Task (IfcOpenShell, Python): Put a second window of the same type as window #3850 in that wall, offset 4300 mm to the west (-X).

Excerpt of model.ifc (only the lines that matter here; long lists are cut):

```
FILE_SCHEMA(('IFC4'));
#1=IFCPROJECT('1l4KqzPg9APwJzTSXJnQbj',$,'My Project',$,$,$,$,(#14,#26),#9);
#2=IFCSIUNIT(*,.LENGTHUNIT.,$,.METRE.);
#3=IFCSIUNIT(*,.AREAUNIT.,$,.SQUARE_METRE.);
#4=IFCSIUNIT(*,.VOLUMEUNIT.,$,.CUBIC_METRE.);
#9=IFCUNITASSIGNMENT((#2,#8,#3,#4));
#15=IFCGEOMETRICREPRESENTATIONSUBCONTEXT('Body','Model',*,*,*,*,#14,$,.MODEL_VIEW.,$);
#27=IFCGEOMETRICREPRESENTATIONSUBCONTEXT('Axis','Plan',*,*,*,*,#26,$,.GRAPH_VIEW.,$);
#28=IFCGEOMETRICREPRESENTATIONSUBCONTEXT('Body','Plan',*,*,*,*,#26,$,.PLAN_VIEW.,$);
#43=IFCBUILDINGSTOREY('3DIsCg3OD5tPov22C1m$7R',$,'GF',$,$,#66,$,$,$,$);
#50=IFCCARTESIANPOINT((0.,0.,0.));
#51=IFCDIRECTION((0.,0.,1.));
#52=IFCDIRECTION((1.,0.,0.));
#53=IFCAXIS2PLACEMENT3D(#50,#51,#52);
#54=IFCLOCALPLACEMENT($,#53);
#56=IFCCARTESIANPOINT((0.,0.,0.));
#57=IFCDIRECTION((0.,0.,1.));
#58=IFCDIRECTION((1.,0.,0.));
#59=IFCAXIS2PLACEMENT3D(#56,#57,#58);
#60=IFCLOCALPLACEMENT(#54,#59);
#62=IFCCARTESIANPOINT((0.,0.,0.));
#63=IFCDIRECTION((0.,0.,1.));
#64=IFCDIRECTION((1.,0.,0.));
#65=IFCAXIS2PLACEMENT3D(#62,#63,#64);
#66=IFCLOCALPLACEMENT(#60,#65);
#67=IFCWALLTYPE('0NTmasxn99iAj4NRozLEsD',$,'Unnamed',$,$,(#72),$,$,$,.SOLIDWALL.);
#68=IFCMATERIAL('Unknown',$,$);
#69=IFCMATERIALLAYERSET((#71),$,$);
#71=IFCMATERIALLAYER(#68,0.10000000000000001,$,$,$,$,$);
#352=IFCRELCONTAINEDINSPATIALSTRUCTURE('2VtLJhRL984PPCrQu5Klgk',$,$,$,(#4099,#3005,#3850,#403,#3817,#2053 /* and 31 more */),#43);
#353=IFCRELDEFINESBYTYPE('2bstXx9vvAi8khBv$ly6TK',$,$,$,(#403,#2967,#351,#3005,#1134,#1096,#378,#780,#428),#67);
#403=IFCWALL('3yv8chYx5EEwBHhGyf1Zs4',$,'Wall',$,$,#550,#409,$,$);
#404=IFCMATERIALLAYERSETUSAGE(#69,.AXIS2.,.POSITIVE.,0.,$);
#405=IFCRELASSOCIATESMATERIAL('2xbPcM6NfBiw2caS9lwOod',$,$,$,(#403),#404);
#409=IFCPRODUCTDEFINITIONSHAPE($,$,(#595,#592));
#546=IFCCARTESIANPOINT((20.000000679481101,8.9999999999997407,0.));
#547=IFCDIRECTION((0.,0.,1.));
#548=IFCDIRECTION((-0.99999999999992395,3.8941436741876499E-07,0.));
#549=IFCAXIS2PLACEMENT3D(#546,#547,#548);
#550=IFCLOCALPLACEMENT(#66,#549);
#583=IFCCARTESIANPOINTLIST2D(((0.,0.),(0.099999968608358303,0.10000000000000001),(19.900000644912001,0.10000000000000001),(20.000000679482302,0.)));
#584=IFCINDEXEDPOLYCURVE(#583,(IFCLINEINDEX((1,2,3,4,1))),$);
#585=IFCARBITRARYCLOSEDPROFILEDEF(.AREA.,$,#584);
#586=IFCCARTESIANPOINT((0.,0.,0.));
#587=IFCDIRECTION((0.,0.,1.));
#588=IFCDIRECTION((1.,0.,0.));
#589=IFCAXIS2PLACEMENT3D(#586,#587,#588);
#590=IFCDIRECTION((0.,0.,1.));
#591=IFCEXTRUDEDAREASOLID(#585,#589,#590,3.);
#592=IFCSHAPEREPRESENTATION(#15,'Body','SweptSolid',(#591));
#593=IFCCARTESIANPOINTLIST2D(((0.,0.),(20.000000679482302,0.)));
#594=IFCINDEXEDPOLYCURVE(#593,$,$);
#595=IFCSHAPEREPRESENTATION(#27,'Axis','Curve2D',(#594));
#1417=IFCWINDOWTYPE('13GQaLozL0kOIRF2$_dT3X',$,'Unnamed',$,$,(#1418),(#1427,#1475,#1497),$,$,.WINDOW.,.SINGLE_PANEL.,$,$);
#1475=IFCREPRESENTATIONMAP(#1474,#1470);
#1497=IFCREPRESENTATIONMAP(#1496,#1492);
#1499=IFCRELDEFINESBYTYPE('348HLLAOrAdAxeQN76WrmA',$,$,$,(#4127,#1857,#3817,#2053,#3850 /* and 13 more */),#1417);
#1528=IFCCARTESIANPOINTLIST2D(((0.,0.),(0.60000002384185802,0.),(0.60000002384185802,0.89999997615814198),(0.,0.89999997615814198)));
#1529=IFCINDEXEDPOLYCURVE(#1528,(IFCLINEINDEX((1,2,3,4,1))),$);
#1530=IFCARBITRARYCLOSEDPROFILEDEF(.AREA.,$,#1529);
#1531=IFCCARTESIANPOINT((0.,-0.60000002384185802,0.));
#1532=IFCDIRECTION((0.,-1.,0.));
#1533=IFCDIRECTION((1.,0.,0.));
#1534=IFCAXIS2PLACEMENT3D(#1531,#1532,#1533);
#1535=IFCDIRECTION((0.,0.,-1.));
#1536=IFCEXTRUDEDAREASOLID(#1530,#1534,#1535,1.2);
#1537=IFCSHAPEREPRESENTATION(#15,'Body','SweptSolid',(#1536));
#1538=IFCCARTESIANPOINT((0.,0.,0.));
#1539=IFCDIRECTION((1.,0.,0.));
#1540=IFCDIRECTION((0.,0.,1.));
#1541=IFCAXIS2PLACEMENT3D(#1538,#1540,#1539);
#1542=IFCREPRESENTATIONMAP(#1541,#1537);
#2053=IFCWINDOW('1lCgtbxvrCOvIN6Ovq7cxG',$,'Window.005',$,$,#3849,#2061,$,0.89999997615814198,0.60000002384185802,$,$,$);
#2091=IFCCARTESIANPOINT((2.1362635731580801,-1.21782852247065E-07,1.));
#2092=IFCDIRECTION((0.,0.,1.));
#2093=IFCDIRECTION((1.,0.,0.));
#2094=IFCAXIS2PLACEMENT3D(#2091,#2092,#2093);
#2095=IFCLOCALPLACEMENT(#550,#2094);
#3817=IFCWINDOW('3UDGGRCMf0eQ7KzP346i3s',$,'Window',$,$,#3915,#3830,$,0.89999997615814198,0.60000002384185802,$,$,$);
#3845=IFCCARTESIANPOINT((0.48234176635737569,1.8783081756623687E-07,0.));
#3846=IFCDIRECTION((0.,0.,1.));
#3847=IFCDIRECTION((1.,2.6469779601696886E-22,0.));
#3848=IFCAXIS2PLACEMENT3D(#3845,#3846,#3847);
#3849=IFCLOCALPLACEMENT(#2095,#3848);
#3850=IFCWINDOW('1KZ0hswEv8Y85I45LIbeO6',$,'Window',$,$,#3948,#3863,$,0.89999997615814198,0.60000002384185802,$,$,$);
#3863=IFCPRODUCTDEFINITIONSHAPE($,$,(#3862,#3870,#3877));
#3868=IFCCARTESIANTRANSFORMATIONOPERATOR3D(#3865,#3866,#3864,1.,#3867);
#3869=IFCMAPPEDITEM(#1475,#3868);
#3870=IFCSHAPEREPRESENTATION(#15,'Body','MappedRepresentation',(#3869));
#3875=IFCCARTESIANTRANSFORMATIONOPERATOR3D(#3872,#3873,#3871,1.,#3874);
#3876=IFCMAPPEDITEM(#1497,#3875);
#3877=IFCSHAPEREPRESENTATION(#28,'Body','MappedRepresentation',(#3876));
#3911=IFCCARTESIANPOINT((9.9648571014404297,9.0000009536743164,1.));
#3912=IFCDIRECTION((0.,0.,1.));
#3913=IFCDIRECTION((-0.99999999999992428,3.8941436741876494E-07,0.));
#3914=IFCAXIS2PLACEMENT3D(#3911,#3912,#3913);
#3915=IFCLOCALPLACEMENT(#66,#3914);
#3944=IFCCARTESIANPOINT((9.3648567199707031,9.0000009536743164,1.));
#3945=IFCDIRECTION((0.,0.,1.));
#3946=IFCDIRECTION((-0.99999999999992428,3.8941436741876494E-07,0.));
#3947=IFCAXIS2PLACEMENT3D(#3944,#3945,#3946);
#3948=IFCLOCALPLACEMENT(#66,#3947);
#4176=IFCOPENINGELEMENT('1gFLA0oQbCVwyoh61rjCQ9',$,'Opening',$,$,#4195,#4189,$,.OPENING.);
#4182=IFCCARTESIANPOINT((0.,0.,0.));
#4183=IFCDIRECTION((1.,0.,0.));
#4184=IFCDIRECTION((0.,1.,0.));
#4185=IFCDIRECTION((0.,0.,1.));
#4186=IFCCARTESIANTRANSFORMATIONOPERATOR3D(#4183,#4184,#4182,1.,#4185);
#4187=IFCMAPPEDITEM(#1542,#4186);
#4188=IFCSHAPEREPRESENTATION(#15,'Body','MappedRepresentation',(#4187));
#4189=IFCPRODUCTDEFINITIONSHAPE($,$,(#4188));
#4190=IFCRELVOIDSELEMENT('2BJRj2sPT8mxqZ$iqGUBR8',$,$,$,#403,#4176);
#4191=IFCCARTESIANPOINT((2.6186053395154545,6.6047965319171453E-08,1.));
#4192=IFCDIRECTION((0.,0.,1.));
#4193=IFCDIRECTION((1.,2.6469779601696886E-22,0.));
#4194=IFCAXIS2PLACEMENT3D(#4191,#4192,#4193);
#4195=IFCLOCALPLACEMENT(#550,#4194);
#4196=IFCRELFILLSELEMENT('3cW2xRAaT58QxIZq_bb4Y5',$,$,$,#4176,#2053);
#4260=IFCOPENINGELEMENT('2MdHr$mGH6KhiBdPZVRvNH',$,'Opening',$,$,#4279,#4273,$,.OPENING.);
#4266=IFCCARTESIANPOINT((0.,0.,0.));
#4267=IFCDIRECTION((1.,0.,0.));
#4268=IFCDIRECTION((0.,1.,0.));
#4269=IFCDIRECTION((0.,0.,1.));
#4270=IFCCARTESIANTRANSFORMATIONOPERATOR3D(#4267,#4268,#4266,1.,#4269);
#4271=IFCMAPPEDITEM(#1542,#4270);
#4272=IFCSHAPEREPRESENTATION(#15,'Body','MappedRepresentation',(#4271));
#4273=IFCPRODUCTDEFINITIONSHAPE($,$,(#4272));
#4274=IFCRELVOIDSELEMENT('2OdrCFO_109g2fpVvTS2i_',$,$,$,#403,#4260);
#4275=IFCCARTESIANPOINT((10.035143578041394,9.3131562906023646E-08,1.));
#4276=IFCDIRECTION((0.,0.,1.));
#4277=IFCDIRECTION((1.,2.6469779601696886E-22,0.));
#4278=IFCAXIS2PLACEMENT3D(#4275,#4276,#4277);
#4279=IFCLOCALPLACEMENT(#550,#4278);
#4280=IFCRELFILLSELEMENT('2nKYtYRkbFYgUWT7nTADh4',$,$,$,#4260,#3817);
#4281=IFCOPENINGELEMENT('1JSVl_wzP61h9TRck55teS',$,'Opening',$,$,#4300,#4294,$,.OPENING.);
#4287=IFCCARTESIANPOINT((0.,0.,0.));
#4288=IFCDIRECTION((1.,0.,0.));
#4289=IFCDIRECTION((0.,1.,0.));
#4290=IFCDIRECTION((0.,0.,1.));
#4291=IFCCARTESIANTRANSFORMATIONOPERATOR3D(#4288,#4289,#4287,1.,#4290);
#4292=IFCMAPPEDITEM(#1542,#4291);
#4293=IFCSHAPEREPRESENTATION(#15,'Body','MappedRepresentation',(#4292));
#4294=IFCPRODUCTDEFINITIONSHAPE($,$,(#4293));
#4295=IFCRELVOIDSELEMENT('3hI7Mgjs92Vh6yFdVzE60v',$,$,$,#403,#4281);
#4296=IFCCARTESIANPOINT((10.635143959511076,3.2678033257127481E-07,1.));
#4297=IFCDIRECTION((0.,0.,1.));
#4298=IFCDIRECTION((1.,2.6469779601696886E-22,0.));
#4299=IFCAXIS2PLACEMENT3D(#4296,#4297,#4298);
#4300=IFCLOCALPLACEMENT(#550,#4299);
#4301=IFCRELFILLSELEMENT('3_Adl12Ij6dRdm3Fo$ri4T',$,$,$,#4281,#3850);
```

```python
import ifcopenshell
import ifcopenshell.api.feature
import ifcopenshell.api.geometry
import ifcopenshell.api.root
import ifcopenshell.geom
import ifcopenshell.util.element
import ifcopenshell.util.placement
import ifcopenshell.util.shape
import ifcopenshell.util.unit

model = ifcopenshell.open("model.ifc")
unit_scale = ifcopenshell.util.unit.calculate_unit_scale(model)
settings = ifcopenshell.geom.settings()


def volume(element):
    """Net volume in cubic metres, openings subtracted."""
    shape = ifcopenshell.geom.create_shape(settings, element)
    return ifcopenshell.util.shape.get_volume(shape.geometry)


window = model.by_guid("1KZ0hswEv8Y85I45LIbeO6")
opening = window.FillsVoids[0].RelatingOpeningElement
wall = opening.VoidsElements[0].RelatingBuildingElement
before = volume(wall)
shift = ifcopenshell.util.placement.get_local_placement(wall.ObjectPlacement)[:3, 0] * 4.3 / unit_scale

# copy_class copies the void relationship, type, container and properties, but no geometry.
new_opening = ifcopenshell.api.root.copy_class(model, product=opening)
new_opening.Representation = ifcopenshell.util.element.copy_deep(
    model, opening.Representation, exclude=["IfcGeometricRepresentationContext", "IfcRepresentationMap"]
)
new_window = ifcopenshell.api.root.copy_class(model, product=window)
new_window.Representation = ifcopenshell.util.element.copy_deep(
    model, window.Representation, exclude=["IfcGeometricRepresentationContext", "IfcRepresentationMap"]
)
ifcopenshell.api.feature.add_filling(model, opening=new_opening, element=new_window)

for old, new in ((opening, new_opening), (window, new_window)):
    matrix = ifcopenshell.util.placement.get_local_placement(old.ObjectPlacement)
    matrix[:3, 3] += shift
    ifcopenshell.api.geometry.edit_object_placement(model, product=new, matrix=matrix, is_si=False)

after = volume(wall)

print(f"wall volume {before:.3f} -> {after:.3f} m3")

model.write("model_rev.ifc")
```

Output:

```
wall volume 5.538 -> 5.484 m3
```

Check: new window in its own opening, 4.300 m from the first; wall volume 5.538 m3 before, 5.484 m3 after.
